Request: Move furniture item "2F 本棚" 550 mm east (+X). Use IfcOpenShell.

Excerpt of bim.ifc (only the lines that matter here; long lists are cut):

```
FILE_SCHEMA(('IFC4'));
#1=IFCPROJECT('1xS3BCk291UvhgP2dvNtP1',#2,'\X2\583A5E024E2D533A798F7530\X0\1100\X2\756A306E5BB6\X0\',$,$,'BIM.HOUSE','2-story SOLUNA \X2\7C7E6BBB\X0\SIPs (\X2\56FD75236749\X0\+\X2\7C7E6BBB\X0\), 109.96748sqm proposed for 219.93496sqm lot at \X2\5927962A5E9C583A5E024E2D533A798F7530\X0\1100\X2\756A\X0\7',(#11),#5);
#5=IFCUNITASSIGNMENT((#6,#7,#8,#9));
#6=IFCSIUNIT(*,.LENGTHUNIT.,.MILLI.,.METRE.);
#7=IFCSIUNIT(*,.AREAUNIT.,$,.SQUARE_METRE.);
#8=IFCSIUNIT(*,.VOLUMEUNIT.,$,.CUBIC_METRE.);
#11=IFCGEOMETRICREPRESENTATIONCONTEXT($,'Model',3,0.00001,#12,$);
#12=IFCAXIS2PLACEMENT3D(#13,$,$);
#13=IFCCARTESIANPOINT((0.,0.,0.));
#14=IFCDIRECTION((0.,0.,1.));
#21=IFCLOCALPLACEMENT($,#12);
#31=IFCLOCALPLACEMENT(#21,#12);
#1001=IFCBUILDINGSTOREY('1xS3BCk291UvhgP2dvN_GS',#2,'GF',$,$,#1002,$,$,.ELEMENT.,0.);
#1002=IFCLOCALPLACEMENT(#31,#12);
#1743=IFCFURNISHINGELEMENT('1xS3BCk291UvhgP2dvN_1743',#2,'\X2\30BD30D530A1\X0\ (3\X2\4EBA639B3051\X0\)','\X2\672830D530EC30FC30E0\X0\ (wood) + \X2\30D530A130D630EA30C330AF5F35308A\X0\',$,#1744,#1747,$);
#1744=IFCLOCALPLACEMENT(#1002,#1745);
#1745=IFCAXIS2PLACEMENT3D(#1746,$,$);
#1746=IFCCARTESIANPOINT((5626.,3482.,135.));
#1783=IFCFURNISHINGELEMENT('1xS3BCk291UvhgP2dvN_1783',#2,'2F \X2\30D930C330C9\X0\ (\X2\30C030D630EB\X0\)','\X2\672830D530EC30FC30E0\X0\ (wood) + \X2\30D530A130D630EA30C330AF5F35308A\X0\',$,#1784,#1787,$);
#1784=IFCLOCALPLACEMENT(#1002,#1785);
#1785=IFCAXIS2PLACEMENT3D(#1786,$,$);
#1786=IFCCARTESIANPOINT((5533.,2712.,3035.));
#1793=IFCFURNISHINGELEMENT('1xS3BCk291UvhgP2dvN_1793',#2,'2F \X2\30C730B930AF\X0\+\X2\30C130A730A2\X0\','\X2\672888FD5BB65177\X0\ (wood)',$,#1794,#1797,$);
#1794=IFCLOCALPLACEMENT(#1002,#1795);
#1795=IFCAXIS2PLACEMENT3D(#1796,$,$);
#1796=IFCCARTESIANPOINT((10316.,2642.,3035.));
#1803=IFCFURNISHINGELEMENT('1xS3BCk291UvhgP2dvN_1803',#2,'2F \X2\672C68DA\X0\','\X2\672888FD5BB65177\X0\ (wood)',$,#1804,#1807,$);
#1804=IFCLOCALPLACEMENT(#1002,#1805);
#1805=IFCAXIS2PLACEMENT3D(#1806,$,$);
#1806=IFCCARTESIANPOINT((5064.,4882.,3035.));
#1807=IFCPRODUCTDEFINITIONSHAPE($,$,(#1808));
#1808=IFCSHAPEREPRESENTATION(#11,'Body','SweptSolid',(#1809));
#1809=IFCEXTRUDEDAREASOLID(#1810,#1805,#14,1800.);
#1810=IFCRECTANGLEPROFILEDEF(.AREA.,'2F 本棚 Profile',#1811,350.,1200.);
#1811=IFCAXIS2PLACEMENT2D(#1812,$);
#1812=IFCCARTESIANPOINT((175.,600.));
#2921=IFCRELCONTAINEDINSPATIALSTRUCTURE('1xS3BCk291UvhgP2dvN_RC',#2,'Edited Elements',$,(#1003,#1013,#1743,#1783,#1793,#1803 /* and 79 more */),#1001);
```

```python
import ifcopenshell
import ifcopenshell.api.geometry
import ifcopenshell.util.placement

model = ifcopenshell.open("bim.ifc")

item = model.by_guid("1xS3BCk291UvhgP2dvN_1803")
matrix = ifcopenshell.util.placement.get_local_placement(item.ObjectPlacement)
matrix[0, 3] += 550.0
ifcopenshell.api.geometry.edit_object_placement(model, product=item, matrix=matrix, is_si=False)

print(ifcopenshell.util.placement.get_local_placement(item.ObjectPlacement).round(3) + 0.0)

model.write("bim-out.ifc")
```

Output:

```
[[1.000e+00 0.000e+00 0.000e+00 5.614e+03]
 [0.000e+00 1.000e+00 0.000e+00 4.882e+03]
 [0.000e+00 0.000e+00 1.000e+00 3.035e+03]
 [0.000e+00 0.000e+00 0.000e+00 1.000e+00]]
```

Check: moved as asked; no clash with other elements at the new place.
